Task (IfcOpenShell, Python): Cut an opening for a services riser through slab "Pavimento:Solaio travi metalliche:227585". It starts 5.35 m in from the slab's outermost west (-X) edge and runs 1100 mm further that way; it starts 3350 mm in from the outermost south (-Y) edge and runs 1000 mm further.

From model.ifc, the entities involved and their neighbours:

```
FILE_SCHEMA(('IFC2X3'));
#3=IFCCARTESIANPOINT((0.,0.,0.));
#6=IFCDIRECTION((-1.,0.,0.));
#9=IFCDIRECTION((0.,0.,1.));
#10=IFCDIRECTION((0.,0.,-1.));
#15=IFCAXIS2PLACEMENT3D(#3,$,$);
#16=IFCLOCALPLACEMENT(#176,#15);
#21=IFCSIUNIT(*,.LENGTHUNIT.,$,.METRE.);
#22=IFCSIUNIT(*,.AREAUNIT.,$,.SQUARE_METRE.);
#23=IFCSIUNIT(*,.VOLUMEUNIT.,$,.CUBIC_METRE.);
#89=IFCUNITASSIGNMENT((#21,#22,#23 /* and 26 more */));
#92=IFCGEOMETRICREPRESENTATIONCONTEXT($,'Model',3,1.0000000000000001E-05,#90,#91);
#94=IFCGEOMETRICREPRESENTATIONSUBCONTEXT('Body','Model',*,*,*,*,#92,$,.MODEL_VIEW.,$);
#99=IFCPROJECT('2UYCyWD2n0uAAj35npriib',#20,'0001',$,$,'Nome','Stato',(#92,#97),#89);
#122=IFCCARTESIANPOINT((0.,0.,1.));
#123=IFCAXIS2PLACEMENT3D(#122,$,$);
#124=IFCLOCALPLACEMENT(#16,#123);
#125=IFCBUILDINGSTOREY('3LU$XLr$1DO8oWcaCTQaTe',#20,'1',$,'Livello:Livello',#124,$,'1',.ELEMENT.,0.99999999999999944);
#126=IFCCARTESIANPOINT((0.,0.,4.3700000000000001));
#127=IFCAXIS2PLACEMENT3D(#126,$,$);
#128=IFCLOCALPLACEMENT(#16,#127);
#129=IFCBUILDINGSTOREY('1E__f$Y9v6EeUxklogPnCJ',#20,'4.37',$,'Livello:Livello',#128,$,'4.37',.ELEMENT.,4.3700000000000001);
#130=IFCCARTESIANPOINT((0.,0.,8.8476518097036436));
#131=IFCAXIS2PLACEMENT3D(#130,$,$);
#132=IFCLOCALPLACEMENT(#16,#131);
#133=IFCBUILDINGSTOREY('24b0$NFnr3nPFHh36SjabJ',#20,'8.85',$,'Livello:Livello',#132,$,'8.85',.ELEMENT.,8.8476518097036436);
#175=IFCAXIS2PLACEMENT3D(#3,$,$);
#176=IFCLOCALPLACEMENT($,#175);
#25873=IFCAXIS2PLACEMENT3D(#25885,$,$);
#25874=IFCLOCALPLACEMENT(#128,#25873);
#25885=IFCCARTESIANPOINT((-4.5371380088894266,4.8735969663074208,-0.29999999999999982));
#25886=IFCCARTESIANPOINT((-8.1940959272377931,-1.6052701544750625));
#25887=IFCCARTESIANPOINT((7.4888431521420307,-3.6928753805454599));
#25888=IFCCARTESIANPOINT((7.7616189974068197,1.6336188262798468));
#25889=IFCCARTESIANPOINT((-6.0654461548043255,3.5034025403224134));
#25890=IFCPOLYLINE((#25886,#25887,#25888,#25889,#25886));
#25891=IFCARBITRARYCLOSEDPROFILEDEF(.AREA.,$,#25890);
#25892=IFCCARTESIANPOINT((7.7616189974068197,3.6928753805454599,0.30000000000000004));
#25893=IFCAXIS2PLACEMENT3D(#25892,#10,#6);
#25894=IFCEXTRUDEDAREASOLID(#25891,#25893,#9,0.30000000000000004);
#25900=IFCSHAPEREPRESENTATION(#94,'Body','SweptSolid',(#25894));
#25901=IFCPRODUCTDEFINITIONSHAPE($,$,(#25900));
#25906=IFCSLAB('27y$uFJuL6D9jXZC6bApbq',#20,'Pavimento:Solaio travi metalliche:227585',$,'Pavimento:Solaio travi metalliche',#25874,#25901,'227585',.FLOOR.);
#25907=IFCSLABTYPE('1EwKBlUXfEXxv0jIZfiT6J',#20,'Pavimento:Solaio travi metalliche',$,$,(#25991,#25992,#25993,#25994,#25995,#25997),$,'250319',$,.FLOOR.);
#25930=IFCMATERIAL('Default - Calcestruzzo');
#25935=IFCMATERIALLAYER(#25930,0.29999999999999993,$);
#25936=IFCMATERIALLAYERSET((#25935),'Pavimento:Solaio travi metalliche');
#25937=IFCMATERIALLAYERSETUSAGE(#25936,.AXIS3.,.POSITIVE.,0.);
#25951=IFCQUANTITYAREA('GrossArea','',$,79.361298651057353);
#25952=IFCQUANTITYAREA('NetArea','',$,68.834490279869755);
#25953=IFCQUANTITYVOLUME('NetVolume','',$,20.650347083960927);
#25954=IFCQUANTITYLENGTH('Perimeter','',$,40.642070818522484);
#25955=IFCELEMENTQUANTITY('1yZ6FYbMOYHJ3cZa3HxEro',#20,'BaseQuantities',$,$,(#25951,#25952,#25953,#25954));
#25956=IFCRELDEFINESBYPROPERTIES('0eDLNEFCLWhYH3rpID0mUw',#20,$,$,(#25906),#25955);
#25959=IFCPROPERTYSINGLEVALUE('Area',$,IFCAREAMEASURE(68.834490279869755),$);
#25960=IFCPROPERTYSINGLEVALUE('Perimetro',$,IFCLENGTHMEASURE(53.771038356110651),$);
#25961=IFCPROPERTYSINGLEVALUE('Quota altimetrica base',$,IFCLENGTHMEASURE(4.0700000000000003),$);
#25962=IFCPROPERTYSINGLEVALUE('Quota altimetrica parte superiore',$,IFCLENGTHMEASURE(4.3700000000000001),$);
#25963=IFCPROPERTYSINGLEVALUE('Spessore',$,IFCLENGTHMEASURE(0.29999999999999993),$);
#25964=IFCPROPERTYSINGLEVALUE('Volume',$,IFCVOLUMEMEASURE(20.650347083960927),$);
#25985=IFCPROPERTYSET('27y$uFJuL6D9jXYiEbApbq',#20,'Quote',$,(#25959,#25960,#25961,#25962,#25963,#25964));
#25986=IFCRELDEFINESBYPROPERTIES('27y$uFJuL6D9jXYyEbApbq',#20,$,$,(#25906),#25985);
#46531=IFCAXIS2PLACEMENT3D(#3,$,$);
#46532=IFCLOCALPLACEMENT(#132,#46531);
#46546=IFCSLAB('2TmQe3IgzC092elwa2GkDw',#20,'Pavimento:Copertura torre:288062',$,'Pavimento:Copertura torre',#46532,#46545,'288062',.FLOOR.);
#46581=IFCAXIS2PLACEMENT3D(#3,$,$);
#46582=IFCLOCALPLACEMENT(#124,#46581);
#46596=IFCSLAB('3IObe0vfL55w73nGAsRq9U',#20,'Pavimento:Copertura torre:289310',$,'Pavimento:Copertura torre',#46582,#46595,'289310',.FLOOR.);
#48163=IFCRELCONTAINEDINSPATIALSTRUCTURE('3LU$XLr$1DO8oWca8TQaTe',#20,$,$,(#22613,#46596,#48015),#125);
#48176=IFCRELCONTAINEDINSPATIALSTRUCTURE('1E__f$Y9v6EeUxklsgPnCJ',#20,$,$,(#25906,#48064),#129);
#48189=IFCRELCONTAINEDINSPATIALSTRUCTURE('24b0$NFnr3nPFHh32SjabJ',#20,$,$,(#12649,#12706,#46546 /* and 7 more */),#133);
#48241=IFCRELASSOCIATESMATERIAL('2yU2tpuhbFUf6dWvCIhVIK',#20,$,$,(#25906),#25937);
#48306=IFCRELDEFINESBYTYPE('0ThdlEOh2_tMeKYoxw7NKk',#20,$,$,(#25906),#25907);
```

```python
import numpy as np
import ifcopenshell
import ifcopenshell.api.feature
import ifcopenshell.api.geometry
import ifcopenshell.api.pset
import ifcopenshell.api.root
import ifcopenshell.geom
import ifcopenshell.util.element
import ifcopenshell.util.placement
import ifcopenshell.util.representation
import ifcopenshell.util.shape
import ifcopenshell.util.unit

model = ifcopenshell.open("model.ifc")
unit_scale = ifcopenshell.util.unit.calculate_unit_scale(model)
area_scale = ifcopenshell.util.unit.calculate_unit_scale(model, "AREAUNIT")
volume_scale = ifcopenshell.util.unit.calculate_unit_scale(model, "VOLUMEUNIT")
settings = ifcopenshell.geom.settings()


def volume(element):
    """Net volume in cubic metres, openings subtracted."""
    shape = ifcopenshell.geom.create_shape(settings, element)
    return ifcopenshell.util.shape.get_volume(shape.geometry)


slab = model.by_guid("27y$uFJuL6D9jXZC6bApbq")
before = volume(slab)

# Extent in the slab's own axes, in metres. The edges named are its -X and -Y sides.
slab_shape = ifcopenshell.geom.create_shape(settings, slab)
vertices = ifcopenshell.util.shape.get_vertices(slab_shape.geometry)
x_min, y_min, bottom = vertices.min(axis=0)
top = vertices[:, 2].max()

opening = ifcopenshell.api.root.create_entity(model, ifc_class="IfcOpeningElement", name="Services riser opening")
context = ifcopenshell.util.representation.get_context(model, "Model", "Body", "MODEL_VIEW")
width, depth = 1.1, 1
outline = [(0.0, 0.0), (width, 0.0), (width, depth), (0.0, depth), (0.0, 0.0)]
# Overshoot both faces by 50 mm so the cut is clean.
shape = ifcopenshell.api.geometry.add_slab_representation(
    model, context=context, depth=top - bottom + 0.1, polyline=outline
)
ifcopenshell.api.geometry.assign_representation(model, product=opening, representation=shape)

matrix = ifcopenshell.util.placement.get_local_placement(slab.ObjectPlacement)
matrix[:, 3] = matrix @ np.append(np.array([x_min + 5.35, y_min + 3.35, bottom - 0.05]) / unit_scale, 1.0)
ifcopenshell.api.geometry.edit_object_placement(model, product=opening, matrix=matrix, is_si=False)
ifcopenshell.api.feature.add_feature(model, feature=opening, element=slab)

after = volume(slab)

# Update the slab's stored quantities.
qto = model.by_id(ifcopenshell.util.element.get_pset(slab, "BaseQuantities", should_inherit=False)["id"])
ifcopenshell.api.pset.edit_qto(model, qto=qto, properties={
    "NetArea": after / (top - bottom) / area_scale,
    "NetVolume": after / volume_scale,
})
pset = model.by_id(ifcopenshell.util.element.get_pset(slab, "Quote", should_inherit=False)["id"])
ifcopenshell.api.pset.edit_pset(model, pset=pset, properties={
    "Area": model.create_entity("IfcAreaMeasure", after / (top - bottom) / area_scale),
    "Volume": model.create_entity("IfcVolumeMeasure", after / volume_scale),
})

print(f"slab volume {before:.3f} -> {after:.3f} m3")

model.write("model-out.ifc")
```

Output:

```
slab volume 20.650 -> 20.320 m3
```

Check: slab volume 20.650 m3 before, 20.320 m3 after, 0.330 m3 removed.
